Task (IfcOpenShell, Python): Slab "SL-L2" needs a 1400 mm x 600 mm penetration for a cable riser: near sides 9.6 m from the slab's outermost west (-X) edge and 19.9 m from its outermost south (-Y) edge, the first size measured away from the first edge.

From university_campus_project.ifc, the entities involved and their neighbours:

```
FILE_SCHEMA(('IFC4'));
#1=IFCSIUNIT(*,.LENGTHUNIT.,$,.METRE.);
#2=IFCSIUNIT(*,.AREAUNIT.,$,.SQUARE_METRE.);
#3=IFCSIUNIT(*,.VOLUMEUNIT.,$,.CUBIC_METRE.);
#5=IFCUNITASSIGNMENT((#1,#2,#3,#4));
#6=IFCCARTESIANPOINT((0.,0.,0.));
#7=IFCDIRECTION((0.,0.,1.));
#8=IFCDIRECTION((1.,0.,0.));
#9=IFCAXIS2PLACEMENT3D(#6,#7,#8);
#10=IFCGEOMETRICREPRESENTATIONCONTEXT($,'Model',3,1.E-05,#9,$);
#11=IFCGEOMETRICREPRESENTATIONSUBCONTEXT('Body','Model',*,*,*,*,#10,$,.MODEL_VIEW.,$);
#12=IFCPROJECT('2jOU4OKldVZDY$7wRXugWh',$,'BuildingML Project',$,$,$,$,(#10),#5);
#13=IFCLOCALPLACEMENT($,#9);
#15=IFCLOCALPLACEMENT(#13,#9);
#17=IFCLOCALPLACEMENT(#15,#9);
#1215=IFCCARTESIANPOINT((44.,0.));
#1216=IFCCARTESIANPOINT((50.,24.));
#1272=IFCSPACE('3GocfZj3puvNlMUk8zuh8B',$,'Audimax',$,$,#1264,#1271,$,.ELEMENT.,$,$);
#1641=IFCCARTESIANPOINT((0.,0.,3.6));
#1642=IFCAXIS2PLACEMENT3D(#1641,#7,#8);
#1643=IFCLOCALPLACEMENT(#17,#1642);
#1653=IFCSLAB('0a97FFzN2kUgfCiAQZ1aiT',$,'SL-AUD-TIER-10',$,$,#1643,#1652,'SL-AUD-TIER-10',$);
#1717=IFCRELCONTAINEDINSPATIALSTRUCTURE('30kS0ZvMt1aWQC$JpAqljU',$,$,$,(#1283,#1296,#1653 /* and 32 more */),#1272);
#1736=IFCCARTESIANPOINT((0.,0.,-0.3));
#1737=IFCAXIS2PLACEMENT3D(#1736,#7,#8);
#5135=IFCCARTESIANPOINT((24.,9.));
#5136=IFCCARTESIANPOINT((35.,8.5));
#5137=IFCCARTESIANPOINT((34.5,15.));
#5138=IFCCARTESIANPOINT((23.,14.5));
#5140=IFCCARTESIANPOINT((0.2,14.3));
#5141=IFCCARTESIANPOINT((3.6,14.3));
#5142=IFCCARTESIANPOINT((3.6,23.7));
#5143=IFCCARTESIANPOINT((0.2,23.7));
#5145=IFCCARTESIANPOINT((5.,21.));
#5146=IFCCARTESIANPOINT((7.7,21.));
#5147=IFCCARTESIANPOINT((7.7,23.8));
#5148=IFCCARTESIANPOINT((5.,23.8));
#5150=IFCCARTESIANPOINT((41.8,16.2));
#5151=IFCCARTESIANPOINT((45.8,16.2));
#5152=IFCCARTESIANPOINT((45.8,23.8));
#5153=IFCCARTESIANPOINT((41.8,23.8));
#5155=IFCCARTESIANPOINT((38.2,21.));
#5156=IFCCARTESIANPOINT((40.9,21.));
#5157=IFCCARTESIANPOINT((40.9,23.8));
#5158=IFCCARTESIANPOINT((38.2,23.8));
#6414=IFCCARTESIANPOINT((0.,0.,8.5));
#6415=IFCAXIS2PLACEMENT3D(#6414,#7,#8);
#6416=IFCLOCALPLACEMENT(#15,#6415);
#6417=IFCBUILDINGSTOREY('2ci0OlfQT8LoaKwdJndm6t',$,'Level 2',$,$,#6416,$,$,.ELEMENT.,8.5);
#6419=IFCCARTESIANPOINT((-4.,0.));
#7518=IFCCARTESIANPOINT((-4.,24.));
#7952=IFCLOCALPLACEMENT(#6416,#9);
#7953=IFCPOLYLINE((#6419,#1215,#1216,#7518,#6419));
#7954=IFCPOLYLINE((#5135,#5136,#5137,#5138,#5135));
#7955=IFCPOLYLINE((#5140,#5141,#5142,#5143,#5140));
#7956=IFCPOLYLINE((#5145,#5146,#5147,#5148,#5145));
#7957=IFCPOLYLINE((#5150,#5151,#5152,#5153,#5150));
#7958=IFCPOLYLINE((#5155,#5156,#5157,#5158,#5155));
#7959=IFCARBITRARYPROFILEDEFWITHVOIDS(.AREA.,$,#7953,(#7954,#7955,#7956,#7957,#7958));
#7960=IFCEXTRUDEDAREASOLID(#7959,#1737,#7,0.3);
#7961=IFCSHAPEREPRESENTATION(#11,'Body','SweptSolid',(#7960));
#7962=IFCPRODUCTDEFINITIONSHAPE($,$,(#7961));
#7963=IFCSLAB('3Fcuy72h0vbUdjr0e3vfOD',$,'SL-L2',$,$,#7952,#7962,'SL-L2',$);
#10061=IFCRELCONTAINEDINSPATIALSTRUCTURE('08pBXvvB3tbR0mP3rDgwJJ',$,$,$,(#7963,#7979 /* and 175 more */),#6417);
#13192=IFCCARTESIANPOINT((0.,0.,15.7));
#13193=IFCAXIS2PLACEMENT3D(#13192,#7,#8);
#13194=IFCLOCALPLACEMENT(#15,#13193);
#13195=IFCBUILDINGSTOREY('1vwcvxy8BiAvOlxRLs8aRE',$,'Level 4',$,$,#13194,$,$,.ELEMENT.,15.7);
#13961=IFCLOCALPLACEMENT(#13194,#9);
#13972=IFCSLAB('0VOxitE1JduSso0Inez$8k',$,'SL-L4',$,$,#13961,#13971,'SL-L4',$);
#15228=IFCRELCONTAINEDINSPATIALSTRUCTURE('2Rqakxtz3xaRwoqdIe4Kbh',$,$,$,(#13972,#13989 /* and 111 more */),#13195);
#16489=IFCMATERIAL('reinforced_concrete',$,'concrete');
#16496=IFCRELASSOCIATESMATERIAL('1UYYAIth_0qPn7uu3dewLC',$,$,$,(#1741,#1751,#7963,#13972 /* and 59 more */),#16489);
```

```python
import numpy as np
import ifcopenshell
import ifcopenshell.api.feature
import ifcopenshell.api.geometry
import ifcopenshell.api.root
import ifcopenshell.geom
import ifcopenshell.util.placement
import ifcopenshell.util.representation
import ifcopenshell.util.shape
import ifcopenshell.util.unit

model = ifcopenshell.open("university_campus_project.ifc")
unit_scale = ifcopenshell.util.unit.calculate_unit_scale(model)
settings = ifcopenshell.geom.settings()


def volume(element):
    """Net volume in cubic metres, openings subtracted."""
    shape = ifcopenshell.geom.create_shape(settings, element)
    return ifcopenshell.util.shape.get_volume(shape.geometry)


slab = model.by_guid("3Fcuy72h0vbUdjr0e3vfOD")
before = volume(slab)

# Extent in the slab's own axes, in metres. The edges named are its -X and -Y sides.
slab_shape = ifcopenshell.geom.create_shape(settings, slab)
vertices = ifcopenshell.util.shape.get_vertices(slab_shape.geometry)
x_min, y_min, bottom = vertices.min(axis=0)
top = vertices[:, 2].max()

opening = ifcopenshell.api.root.create_entity(model, ifc_class="IfcOpeningElement", name="Cable riser opening", predefined_type="OPENING")
context = ifcopenshell.util.representation.get_context(model, "Model", "Body", "MODEL_VIEW")
width, depth = 1.4, 0.6
outline = [(0.0, 0.0), (width, 0.0), (width, depth), (0.0, depth), (0.0, 0.0)]
# Overshoot both faces by 50 mm so the cut is clean.
shape = ifcopenshell.api.geometry.add_slab_representation(
    model, context=context, depth=top - bottom + 0.1, polyline=outline
)
ifcopenshell.api.geometry.assign_representation(model, product=opening, representation=shape)

matrix = ifcopenshell.util.placement.get_local_placement(slab.ObjectPlacement)
matrix[:, 3] = matrix @ np.append(np.array([x_min + 9.6, y_min + 19.9, bottom - 0.05]) / unit_scale, 1.0)
ifcopenshell.api.geometry.edit_object_placement(model, product=opening, matrix=matrix, is_si=False)
ifcopenshell.api.feature.add_feature(model, feature=opening, element=slab)

after = volume(slab)

print(f"slab volume {before:.3f} -> {after:.3f} m3")

model.write("university_campus_project-out.ifc")
```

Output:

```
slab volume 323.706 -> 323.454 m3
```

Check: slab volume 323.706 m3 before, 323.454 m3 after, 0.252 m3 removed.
